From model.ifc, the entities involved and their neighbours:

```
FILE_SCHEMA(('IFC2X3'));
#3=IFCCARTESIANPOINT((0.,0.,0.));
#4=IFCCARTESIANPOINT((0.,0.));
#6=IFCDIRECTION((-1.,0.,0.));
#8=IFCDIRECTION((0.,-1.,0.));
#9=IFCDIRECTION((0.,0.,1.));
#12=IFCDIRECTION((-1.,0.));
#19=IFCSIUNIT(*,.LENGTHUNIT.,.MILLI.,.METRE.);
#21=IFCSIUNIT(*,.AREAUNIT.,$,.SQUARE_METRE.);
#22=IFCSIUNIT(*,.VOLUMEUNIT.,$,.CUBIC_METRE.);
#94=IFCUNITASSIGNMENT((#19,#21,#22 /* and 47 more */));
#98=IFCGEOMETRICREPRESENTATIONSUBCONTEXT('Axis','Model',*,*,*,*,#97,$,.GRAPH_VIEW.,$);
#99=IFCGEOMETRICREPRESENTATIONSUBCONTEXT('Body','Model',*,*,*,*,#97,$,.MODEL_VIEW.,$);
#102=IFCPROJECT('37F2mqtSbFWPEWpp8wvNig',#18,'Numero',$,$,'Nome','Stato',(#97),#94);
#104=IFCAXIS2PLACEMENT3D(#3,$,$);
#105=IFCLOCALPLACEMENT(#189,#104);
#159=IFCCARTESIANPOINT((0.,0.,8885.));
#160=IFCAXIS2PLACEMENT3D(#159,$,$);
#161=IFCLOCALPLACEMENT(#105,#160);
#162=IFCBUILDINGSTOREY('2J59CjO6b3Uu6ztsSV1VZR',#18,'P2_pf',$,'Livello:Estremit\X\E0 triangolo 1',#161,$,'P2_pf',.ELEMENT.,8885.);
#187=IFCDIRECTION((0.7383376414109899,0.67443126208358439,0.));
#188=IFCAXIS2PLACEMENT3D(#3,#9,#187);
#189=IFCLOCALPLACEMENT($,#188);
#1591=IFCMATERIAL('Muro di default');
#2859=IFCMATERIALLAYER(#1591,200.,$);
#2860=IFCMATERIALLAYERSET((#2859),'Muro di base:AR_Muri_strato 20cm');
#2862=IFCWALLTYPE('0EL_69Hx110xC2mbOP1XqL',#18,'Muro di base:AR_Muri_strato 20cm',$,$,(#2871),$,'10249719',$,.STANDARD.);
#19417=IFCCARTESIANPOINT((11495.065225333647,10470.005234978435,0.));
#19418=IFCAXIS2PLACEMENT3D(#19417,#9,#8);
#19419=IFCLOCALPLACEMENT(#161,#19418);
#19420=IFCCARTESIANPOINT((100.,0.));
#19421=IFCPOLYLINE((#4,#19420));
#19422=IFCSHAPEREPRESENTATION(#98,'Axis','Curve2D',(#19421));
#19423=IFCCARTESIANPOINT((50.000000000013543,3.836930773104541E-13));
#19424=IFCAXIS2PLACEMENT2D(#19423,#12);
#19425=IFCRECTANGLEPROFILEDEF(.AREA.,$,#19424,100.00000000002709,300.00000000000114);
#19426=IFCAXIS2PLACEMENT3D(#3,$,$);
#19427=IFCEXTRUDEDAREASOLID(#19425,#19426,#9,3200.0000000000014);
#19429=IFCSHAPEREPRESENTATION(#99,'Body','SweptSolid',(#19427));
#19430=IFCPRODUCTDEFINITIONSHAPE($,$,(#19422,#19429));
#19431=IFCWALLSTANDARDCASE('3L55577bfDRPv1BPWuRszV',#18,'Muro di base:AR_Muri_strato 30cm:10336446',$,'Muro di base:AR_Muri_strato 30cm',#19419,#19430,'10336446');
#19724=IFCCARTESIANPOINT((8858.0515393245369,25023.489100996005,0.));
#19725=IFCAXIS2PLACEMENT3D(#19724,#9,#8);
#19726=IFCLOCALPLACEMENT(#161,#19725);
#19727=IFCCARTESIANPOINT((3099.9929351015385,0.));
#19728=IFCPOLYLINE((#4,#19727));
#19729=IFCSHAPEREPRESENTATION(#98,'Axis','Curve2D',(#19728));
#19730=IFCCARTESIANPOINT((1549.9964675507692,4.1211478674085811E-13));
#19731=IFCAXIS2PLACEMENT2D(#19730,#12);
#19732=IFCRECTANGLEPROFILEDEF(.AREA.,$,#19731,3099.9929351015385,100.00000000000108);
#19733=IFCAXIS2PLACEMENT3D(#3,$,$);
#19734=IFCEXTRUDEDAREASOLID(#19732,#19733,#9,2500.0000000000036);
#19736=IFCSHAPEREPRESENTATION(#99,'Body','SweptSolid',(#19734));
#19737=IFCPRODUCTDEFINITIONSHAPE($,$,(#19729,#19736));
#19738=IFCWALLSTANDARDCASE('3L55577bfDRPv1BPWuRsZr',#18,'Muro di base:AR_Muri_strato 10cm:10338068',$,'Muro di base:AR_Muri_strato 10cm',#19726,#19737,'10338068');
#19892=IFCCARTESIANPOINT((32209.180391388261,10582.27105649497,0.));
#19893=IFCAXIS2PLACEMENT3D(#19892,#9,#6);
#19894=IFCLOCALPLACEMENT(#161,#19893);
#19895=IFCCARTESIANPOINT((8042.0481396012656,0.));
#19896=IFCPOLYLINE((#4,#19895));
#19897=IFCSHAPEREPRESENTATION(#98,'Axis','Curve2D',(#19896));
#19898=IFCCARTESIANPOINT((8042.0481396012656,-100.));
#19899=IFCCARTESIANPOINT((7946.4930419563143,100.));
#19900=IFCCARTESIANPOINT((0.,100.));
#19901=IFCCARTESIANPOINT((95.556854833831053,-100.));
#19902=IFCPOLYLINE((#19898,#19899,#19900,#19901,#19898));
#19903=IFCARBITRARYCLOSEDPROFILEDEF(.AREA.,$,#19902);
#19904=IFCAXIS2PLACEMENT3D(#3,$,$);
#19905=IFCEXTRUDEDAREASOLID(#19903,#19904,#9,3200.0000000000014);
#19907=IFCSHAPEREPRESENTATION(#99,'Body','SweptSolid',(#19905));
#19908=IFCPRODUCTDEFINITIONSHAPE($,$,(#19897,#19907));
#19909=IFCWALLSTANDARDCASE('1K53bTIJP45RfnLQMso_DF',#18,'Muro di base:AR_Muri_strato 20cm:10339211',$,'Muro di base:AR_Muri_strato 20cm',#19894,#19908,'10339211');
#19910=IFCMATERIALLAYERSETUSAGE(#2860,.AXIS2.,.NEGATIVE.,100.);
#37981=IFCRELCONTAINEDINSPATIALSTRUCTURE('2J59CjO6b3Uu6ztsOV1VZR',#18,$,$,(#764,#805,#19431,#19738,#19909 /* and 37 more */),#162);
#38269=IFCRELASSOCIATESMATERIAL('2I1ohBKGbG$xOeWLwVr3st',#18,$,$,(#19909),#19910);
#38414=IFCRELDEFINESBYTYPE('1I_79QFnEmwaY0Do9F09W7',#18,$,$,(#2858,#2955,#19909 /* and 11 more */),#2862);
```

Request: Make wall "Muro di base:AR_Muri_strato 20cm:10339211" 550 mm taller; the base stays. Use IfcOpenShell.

```python
import ifcopenshell
import ifcopenshell.geom
import ifcopenshell.util.representation
import ifcopenshell.util.shape
import ifcopenshell.util.unit

model = ifcopenshell.open("model.ifc")
unit_scale = ifcopenshell.util.unit.calculate_unit_scale(model)
settings = ifcopenshell.geom.settings()


def volume(element):
    """Net volume in cubic metres, openings subtracted."""
    shape = ifcopenshell.geom.create_shape(settings, element)
    return ifcopenshell.util.shape.get_volume(shape.geometry)


wall = model.by_guid("1K53bTIJP45RfnLQMso_DF")
before = volume(wall)

body = ifcopenshell.util.representation.get_representation(wall, "Model", "Body")
solid = body.Items[0]
old_height = solid.Depth
solid.Depth += 0.55 / unit_scale
after = volume(wall)

print(f"height {old_height:g} -> {solid.Depth:g}, volume {before:.3f} -> {after:.3f} m3")

model.write("model-out.ifc")
```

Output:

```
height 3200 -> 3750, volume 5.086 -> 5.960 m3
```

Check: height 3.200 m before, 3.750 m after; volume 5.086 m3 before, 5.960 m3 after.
